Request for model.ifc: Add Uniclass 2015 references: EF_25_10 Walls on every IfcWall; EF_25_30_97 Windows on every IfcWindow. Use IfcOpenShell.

First a look at what the model holds.

```python
import ifcopenshell

model = ifcopenshell.open("model.ifc")
print(model.schema)
print("classifications:", [c.Name for c in model.by_type("IfcClassification")])
for ifc_class in ("IfcDoor", "IfcRoof", "IfcStair", "IfcWall", "IfcWindow"):
    print(ifc_class, len(model.by_type(ifc_class)))
```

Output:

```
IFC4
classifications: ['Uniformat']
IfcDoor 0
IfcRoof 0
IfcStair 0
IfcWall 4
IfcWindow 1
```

```python
import ifcopenshell
import ifcopenshell.api.classification

model = ifcopenshell.open("model.ifc")

system = ifcopenshell.api.classification.add_classification(model, classification="Uniclass 2015")

codes = {
    "IfcWall": ("EF_25_10", "Walls"),
    "IfcWindow": ("EF_25_30_97", "Windows"),
}
for ifc_class, (code, name) in codes.items():
    products = model.by_type(ifc_class)
    ifcopenshell.api.classification.add_reference(
        model, products=products, classification=system, identification=code, name=name
    )
    print(code, len(products))

model.write("model_updated.ifc")
```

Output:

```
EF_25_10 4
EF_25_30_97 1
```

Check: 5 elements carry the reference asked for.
